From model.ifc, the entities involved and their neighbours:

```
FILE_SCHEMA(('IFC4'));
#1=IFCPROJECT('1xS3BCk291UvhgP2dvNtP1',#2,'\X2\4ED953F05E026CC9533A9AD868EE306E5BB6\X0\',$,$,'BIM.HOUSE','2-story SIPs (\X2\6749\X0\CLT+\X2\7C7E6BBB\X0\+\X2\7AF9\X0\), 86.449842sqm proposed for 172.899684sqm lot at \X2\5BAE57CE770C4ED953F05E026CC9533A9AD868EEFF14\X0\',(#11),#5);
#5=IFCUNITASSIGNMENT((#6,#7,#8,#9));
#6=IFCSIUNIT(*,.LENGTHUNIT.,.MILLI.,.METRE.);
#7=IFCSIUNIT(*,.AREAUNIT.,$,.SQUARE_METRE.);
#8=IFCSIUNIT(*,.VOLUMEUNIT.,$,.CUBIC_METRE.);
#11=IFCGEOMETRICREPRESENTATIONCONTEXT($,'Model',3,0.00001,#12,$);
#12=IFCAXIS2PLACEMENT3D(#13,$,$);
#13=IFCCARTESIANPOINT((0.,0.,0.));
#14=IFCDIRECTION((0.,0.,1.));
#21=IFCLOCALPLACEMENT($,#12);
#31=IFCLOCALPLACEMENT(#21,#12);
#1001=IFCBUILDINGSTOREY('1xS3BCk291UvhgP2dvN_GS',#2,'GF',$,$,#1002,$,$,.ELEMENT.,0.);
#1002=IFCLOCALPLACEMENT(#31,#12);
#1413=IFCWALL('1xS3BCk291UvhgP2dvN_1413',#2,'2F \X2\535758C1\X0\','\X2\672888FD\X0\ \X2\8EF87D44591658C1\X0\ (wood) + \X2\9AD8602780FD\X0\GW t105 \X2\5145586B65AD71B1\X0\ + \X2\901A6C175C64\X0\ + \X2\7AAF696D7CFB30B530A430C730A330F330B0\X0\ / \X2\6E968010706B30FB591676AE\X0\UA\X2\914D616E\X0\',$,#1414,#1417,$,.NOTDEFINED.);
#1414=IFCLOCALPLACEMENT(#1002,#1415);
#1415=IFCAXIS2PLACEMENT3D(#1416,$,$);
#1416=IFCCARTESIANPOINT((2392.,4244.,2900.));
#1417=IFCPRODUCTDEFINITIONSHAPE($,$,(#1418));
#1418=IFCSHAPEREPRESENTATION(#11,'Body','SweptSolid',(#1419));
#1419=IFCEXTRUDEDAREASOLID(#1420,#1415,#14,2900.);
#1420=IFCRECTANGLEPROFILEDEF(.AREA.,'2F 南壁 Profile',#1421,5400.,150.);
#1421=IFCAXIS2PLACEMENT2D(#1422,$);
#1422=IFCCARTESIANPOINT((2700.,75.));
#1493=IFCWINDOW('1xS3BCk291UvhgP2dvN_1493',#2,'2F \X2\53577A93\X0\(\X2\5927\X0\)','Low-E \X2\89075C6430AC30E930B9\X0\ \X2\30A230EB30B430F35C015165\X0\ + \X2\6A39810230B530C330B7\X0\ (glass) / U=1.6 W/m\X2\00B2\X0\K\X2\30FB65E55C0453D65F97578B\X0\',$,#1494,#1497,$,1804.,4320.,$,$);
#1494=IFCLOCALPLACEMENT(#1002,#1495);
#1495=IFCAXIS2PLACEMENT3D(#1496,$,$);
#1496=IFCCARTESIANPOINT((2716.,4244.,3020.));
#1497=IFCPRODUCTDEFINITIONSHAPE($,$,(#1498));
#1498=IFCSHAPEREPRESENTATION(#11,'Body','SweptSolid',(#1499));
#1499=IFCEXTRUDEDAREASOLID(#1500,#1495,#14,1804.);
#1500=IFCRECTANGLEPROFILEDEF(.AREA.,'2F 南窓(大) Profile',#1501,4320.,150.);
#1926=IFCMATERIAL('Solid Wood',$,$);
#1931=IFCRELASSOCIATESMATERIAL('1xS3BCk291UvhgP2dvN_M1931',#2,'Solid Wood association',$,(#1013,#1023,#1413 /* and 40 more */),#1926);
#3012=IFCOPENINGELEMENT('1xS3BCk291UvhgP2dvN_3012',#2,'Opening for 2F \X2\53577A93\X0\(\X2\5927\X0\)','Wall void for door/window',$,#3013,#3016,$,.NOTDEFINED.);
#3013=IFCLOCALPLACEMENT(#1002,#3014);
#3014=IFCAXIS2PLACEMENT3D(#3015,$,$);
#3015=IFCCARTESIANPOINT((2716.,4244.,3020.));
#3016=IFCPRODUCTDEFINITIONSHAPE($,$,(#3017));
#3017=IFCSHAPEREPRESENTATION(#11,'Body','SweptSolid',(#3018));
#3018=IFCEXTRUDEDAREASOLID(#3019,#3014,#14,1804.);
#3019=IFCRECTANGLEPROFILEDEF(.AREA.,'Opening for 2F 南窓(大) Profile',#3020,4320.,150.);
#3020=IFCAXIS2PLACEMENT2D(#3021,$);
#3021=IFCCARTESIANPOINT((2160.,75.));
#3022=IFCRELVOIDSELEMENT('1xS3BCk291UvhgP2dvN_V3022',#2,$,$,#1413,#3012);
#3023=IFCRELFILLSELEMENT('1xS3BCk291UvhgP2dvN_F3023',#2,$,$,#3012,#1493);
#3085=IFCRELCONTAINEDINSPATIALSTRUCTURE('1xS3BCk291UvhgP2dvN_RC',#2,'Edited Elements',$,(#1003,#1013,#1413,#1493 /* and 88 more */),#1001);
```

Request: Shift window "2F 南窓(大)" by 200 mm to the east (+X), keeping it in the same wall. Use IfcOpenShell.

```python
import ifcopenshell
import ifcopenshell.api.geometry
import ifcopenshell.util.placement
import ifcopenshell.util.unit

model = ifcopenshell.open("model.ifc")
unit_scale = ifcopenshell.util.unit.calculate_unit_scale(model)

window = model.by_guid("1xS3BCk291UvhgP2dvN_1493")
opening = window.FillsVoids[0].RelatingOpeningElement
wall = opening.VoidsElements[0].RelatingBuildingElement

wall_matrix = ifcopenshell.util.placement.get_local_placement(wall.ObjectPlacement)
shift = wall_matrix[:3, 0] * 0.2 / unit_scale
before = ifcopenshell.util.placement.get_local_placement(window.ObjectPlacement)[:3, 3].copy()

# The window is not placed relative to its opening, so move both.
for product in (opening, window):
    matrix = ifcopenshell.util.placement.get_local_placement(product.ObjectPlacement)
    matrix[:3, 3] += shift
    ifcopenshell.api.geometry.edit_object_placement(model, product=product, matrix=matrix, is_si=False)

after = ifcopenshell.util.placement.get_local_placement(window.ObjectPlacement)[:3, 3]
print("window moved by", (after - before).round(3) + 0.0)

model.write("model_rev.ifc")
```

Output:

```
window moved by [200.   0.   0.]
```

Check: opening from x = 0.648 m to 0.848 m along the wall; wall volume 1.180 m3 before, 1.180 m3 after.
